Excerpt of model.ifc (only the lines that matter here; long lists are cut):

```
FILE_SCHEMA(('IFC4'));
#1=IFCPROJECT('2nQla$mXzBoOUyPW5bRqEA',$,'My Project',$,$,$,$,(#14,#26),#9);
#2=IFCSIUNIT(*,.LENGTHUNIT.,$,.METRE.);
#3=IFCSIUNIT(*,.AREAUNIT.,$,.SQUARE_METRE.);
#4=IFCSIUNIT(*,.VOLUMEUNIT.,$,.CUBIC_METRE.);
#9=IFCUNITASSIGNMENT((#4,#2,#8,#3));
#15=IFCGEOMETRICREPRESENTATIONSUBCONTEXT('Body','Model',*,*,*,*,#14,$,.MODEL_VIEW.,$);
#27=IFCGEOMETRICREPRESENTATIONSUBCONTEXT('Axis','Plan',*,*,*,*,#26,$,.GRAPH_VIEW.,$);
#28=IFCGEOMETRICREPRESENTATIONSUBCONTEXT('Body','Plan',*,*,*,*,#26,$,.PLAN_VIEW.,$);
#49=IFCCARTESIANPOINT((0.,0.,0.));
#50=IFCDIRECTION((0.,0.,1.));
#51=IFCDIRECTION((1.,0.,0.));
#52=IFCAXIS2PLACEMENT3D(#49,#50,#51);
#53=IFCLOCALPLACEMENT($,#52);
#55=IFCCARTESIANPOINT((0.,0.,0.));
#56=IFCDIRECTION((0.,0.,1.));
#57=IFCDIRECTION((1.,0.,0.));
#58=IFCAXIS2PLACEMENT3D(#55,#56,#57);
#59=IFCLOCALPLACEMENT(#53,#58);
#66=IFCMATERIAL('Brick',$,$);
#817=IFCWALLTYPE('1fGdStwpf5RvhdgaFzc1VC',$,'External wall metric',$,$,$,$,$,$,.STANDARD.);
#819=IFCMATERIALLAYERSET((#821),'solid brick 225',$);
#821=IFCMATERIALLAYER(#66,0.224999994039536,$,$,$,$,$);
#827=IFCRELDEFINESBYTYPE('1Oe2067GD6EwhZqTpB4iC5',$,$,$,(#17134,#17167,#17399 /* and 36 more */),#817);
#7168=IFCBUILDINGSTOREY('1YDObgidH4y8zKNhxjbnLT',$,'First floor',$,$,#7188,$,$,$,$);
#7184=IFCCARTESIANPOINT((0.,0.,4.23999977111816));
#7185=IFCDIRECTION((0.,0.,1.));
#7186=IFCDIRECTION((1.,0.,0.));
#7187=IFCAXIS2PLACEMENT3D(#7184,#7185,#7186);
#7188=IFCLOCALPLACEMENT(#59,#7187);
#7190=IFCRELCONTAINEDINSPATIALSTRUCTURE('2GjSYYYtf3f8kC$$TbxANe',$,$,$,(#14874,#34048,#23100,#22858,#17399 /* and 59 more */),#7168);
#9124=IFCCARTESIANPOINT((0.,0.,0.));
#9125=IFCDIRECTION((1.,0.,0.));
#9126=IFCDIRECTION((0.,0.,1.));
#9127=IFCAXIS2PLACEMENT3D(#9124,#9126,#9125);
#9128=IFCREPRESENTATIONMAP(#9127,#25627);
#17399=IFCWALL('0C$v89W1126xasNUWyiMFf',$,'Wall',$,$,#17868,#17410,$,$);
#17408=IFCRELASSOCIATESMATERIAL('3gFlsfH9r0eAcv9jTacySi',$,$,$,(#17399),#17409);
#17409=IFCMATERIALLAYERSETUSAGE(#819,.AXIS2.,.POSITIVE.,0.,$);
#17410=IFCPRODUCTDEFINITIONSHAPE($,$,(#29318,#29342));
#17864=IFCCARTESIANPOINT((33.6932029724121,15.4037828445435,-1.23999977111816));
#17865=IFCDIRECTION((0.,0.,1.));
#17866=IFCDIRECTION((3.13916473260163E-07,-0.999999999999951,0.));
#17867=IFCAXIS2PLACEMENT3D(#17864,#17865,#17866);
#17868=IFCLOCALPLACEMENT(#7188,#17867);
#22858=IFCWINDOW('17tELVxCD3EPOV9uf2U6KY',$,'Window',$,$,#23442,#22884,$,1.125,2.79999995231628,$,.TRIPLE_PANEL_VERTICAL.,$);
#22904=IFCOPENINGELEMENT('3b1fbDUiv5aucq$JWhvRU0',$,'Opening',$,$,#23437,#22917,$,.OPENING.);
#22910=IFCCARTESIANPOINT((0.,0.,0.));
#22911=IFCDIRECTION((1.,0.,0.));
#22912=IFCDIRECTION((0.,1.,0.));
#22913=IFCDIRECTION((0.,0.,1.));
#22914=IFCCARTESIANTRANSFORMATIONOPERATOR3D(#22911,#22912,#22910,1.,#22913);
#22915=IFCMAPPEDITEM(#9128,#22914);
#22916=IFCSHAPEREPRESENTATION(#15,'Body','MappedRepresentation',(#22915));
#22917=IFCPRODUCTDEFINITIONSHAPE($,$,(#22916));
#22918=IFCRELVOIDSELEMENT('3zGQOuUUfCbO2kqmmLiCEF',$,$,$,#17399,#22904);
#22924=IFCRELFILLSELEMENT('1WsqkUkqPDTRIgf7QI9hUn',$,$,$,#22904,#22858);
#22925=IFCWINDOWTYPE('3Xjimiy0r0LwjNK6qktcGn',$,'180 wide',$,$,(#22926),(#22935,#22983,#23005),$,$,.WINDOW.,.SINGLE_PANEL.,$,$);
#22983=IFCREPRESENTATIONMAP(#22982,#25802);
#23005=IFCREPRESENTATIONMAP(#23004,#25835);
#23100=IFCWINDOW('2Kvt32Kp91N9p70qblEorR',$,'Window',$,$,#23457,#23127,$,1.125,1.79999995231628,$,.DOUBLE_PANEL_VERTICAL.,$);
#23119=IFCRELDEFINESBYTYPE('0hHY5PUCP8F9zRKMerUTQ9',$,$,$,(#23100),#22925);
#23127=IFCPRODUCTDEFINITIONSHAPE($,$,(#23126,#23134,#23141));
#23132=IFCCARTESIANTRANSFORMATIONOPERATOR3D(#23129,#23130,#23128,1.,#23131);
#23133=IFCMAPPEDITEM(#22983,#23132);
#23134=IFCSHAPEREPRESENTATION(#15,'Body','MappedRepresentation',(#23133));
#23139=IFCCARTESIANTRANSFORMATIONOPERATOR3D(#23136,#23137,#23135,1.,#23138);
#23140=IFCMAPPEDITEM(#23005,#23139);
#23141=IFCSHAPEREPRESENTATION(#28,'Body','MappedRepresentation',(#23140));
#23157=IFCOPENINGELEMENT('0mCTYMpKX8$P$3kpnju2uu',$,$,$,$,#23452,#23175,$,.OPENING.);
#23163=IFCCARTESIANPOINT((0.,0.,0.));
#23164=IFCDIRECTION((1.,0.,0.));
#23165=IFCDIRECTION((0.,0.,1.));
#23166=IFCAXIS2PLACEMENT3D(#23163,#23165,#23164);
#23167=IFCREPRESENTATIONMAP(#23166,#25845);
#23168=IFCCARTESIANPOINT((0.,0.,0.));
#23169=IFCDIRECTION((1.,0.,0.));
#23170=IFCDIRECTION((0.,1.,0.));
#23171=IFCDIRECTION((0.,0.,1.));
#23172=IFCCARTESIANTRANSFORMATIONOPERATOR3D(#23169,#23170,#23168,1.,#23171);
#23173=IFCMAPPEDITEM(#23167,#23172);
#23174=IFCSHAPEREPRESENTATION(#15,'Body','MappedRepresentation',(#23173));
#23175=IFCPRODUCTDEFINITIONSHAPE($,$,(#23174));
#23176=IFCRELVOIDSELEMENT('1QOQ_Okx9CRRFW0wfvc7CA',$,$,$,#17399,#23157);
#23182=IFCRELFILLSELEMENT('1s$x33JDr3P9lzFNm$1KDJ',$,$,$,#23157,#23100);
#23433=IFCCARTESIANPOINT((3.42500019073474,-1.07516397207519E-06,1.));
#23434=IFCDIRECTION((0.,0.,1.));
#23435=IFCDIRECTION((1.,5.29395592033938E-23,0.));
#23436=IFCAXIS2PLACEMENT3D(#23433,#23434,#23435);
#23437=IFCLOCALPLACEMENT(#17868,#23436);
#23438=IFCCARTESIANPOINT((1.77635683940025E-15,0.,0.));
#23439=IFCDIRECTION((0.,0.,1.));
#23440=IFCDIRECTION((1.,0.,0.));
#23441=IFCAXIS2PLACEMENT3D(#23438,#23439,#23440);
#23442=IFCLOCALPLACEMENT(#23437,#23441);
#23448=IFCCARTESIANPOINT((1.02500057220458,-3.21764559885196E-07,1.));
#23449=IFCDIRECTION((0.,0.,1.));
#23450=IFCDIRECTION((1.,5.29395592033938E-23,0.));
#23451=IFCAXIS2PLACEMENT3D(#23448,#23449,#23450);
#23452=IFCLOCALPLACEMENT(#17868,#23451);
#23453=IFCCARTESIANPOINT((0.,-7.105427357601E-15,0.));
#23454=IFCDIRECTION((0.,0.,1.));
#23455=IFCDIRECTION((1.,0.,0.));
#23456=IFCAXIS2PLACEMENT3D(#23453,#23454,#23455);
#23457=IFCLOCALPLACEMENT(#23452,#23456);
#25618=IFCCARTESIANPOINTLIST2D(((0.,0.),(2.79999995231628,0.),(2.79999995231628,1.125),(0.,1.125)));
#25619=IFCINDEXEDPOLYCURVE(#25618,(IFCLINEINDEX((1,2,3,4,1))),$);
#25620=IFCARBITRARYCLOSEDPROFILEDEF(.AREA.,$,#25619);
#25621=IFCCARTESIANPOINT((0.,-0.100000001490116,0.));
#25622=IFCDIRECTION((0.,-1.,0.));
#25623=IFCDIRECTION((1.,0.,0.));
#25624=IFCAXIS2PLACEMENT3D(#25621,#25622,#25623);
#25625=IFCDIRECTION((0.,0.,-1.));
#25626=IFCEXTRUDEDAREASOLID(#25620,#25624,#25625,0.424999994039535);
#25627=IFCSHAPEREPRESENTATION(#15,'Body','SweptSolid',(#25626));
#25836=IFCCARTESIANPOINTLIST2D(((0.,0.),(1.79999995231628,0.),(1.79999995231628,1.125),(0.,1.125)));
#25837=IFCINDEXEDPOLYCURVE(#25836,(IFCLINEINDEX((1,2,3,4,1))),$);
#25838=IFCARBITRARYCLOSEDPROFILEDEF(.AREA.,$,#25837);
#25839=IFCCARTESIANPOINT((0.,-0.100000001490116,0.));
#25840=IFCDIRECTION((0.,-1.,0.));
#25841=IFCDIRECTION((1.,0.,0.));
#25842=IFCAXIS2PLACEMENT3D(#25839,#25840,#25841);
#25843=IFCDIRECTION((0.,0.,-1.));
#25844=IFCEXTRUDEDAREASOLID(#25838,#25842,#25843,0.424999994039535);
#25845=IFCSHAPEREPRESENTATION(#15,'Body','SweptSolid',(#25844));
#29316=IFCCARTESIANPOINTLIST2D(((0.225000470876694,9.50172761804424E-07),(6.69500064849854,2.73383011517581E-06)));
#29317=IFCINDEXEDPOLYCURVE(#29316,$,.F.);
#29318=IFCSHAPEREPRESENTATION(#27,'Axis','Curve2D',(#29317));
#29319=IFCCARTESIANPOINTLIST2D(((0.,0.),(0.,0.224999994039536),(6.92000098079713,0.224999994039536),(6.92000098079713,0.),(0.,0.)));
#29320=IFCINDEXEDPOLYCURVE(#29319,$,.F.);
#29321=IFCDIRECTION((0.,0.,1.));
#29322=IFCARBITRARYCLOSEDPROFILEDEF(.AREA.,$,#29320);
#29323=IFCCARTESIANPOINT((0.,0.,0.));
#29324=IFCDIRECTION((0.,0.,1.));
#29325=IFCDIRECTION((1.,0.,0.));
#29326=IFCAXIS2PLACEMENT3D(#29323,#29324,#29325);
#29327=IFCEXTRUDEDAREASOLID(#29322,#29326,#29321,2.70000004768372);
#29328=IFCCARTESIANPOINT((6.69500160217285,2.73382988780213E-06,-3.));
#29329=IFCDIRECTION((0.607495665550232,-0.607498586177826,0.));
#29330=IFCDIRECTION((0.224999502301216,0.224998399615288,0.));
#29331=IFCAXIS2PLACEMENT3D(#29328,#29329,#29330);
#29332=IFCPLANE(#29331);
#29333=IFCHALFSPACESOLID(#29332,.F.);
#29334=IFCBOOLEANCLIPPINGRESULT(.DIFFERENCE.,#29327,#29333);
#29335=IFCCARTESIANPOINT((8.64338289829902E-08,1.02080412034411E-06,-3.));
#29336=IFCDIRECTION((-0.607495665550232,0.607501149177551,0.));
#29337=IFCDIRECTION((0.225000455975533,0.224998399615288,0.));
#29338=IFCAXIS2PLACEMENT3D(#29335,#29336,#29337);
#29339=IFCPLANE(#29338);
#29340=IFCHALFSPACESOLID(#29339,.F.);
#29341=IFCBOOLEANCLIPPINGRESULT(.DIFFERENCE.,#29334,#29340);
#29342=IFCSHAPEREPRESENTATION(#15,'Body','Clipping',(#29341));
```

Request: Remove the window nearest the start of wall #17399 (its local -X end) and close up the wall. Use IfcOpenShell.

```python
import ifcopenshell
import ifcopenshell.api.feature
import ifcopenshell.api.root
import ifcopenshell.geom
import ifcopenshell.util.shape

model = ifcopenshell.open("model.ifc")
settings = ifcopenshell.geom.settings()


def volume(element):
    """Net volume in cubic metres, openings subtracted."""
    shape = ifcopenshell.geom.create_shape(settings, element)
    return ifcopenshell.util.shape.get_volume(shape.geometry)


window = model.by_guid("2Kvt32Kp91N9p70qblEorR")
opening = window.FillsVoids[0].RelatingOpeningElement
wall = opening.VoidsElements[0].RelatingBuildingElement
before = volume(wall)

ifcopenshell.api.root.remove_product(model, product=window)
ifcopenshell.api.feature.remove_feature(model, feature=opening)

after = volume(wall)

print(f"wall volume {before:.3f} -> {after:.3f} m3")

model.write("model_updated.ifc")
```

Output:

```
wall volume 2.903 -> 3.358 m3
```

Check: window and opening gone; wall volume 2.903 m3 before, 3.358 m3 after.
